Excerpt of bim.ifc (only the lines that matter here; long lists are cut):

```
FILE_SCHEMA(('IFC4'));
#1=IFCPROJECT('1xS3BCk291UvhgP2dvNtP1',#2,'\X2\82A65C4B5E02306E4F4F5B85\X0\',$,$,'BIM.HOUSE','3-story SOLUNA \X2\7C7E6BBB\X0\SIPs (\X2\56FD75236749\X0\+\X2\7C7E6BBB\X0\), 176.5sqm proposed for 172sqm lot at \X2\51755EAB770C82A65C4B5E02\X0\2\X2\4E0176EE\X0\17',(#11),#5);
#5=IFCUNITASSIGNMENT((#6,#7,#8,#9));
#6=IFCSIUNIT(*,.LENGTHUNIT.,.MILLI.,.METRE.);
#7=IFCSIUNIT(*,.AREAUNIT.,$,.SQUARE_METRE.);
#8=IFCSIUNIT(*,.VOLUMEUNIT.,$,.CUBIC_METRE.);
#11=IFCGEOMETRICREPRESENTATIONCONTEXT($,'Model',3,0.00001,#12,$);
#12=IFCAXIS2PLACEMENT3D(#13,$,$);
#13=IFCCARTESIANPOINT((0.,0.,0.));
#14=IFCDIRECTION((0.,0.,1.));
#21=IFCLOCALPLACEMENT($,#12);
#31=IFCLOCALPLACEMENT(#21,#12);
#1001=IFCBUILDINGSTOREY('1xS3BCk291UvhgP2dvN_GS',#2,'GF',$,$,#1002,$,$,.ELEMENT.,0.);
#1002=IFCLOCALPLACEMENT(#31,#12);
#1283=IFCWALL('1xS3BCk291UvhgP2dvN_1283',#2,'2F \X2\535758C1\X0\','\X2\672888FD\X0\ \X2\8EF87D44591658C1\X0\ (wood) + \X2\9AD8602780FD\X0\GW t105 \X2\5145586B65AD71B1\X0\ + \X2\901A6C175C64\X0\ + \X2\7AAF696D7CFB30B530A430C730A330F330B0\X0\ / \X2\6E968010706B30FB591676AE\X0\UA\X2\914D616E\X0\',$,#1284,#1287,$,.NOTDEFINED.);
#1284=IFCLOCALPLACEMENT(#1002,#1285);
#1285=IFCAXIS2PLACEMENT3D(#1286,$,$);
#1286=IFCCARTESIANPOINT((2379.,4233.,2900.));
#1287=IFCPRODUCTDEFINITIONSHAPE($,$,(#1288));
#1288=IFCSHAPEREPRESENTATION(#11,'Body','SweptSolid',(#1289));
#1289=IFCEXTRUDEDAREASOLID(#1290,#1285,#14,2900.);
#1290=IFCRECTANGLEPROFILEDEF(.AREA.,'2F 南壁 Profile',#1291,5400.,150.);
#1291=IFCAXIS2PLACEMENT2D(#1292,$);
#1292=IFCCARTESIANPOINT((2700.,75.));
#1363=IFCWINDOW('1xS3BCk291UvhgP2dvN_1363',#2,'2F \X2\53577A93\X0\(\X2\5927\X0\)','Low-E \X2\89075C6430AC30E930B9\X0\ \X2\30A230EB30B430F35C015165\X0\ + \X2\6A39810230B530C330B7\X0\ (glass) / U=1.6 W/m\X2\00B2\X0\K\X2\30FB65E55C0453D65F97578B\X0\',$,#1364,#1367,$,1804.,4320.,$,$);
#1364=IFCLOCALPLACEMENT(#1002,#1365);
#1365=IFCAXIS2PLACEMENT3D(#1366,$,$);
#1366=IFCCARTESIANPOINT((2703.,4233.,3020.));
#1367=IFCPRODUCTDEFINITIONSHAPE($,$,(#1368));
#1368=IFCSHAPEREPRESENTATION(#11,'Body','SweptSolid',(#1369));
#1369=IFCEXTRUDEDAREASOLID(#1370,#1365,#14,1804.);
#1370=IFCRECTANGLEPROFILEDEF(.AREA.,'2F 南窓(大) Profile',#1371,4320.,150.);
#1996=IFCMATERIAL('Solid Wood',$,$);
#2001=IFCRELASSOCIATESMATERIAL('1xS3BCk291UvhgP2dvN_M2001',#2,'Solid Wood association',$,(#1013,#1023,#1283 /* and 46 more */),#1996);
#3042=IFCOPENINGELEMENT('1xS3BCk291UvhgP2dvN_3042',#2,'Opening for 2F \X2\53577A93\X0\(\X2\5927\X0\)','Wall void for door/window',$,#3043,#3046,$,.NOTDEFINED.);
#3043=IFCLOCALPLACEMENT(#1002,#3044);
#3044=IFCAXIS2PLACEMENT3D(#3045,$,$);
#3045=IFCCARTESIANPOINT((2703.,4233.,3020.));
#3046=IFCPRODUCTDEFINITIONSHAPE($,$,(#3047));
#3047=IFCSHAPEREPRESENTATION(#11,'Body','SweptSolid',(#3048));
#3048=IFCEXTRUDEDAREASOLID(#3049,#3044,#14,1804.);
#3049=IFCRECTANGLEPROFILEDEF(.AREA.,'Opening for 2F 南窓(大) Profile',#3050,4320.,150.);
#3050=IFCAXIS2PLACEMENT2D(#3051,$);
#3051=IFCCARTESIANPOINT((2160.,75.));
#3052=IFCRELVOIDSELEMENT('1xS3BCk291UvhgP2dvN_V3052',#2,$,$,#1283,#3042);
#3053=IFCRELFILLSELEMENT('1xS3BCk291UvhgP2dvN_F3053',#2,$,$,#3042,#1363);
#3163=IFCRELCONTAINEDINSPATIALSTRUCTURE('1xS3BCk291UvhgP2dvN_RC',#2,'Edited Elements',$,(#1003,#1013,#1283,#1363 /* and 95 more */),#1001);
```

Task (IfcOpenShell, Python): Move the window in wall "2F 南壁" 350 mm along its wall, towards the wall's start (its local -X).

```python
import ifcopenshell
import ifcopenshell.api.geometry
import ifcopenshell.util.placement

model = ifcopenshell.open("bim.ifc")

window = model.by_guid("1xS3BCk291UvhgP2dvN_1363")
opening = window.FillsVoids[0].RelatingOpeningElement
wall = opening.VoidsElements[0].RelatingBuildingElement

wall_matrix = ifcopenshell.util.placement.get_local_placement(wall.ObjectPlacement)
shift = wall_matrix[:3, 0] * -350.0
before = ifcopenshell.util.placement.get_local_placement(window.ObjectPlacement)[:3, 3].copy()

# The window is not placed relative to its opening, so move both.
for product in (opening, window):
    matrix = ifcopenshell.util.placement.get_local_placement(product.ObjectPlacement)
    matrix[:3, 3] += shift
    ifcopenshell.api.geometry.edit_object_placement(model, product=product, matrix=matrix, is_si=False)

after = ifcopenshell.util.placement.get_local_placement(window.ObjectPlacement)[:3, 3]
print("window moved by", (after - before).round(3) + 0.0)

model.write("bim_v2.ifc")
```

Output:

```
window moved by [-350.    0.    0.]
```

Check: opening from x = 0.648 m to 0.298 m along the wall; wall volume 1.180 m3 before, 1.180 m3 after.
